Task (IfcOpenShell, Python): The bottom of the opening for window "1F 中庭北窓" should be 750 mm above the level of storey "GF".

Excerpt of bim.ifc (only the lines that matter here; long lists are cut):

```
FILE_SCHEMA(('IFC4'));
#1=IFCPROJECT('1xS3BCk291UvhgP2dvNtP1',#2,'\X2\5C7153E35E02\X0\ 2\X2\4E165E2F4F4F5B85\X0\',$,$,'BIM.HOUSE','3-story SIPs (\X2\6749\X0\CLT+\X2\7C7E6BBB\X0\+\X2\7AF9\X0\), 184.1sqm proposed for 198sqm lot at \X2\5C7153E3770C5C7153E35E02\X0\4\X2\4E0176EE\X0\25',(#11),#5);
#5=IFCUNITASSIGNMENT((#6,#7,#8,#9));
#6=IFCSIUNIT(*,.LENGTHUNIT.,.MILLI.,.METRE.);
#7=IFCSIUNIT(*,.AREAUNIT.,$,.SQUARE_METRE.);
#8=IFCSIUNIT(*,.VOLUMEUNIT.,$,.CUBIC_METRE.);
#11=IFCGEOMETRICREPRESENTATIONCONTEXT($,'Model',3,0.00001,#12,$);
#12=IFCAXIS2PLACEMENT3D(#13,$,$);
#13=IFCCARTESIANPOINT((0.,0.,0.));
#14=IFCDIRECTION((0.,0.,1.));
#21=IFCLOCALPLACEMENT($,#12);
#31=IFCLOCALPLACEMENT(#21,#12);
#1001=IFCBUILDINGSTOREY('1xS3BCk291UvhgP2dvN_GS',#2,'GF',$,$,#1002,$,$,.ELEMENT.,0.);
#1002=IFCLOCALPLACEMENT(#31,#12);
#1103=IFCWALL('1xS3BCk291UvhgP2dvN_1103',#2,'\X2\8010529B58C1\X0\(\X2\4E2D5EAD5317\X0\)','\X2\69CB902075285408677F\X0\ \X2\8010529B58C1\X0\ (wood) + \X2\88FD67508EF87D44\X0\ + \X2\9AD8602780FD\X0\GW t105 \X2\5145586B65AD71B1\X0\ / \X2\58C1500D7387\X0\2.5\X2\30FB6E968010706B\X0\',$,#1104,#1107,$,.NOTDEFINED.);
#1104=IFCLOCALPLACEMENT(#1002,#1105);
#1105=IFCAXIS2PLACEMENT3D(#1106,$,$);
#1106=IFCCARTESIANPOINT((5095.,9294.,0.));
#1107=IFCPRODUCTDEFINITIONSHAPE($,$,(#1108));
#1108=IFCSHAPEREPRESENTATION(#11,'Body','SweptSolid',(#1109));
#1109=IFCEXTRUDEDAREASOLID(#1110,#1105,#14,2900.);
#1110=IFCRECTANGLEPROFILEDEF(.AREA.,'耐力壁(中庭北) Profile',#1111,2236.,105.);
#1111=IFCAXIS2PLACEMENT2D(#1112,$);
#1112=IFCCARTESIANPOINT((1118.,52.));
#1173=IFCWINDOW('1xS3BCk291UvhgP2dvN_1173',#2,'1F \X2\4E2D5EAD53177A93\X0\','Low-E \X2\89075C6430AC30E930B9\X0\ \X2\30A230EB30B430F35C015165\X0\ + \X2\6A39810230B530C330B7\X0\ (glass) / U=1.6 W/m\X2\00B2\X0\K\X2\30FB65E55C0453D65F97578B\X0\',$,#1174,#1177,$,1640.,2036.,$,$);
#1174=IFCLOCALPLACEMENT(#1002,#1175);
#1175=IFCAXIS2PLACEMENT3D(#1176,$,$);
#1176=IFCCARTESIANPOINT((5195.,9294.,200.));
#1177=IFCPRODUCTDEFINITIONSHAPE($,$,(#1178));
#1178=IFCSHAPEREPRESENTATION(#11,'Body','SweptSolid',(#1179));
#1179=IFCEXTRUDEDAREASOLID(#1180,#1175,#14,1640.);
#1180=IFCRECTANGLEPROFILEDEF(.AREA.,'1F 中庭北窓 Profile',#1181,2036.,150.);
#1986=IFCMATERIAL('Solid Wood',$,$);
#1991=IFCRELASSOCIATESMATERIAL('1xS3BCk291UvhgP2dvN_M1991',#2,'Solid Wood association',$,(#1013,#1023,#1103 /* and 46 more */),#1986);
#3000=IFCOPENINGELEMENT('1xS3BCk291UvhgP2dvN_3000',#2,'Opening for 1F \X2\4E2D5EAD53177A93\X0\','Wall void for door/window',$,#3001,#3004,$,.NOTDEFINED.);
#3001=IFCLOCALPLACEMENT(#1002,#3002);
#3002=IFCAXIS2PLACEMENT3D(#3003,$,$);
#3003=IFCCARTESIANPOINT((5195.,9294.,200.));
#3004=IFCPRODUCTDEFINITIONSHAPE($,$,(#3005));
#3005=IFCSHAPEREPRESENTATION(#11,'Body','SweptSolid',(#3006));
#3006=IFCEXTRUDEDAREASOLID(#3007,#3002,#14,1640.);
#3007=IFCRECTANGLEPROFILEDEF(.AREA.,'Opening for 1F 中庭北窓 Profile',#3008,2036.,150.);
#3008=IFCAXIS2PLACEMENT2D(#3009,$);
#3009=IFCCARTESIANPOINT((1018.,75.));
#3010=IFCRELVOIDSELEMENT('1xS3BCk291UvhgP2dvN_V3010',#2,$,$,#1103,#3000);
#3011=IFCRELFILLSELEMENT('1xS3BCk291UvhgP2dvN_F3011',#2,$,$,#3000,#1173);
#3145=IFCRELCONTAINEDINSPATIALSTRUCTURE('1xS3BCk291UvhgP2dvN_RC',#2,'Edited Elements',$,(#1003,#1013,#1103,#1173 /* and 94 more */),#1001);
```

```python
import numpy as np
import ifcopenshell
import ifcopenshell.api.geometry
import ifcopenshell.geom
import ifcopenshell.util.element
import ifcopenshell.util.placement
import ifcopenshell.util.shape
import ifcopenshell.util.unit

model = ifcopenshell.open("bim.ifc")
unit_scale = ifcopenshell.util.unit.calculate_unit_scale(model)

window = model.by_guid("1xS3BCk291UvhgP2dvN_1173")
opening = window.FillsVoids[0].RelatingOpeningElement
storey = ifcopenshell.util.element.get_container(window, ifc_class="IfcBuildingStorey")
level = ifcopenshell.util.placement.get_local_placement(storey.ObjectPlacement)[2, 3]

# The opening's origin need not be at the sill, so measure its lowest point.
shape = ifcopenshell.geom.create_shape(ifcopenshell.geom.settings(), opening)
bottom = ifcopenshell.util.shape.get_shape_bottom_elevation(shape, shape.geometry) / unit_scale
dz = level + 0.75 / unit_scale - bottom

shift = np.array([0.0, 0.0, dz])
# The window is not placed relative to its opening, so move both.
for product in (opening, window):
    matrix = ifcopenshell.util.placement.get_local_placement(product.ObjectPlacement)
    matrix[:3, 3] += shift
    ifcopenshell.api.geometry.edit_object_placement(model, product=product, matrix=matrix, is_si=False)

print(f"moved by {dz * unit_scale:+.3f} m")

model.write("bim_updated.ifc")
```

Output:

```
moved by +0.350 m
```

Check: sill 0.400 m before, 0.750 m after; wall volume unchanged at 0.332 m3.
